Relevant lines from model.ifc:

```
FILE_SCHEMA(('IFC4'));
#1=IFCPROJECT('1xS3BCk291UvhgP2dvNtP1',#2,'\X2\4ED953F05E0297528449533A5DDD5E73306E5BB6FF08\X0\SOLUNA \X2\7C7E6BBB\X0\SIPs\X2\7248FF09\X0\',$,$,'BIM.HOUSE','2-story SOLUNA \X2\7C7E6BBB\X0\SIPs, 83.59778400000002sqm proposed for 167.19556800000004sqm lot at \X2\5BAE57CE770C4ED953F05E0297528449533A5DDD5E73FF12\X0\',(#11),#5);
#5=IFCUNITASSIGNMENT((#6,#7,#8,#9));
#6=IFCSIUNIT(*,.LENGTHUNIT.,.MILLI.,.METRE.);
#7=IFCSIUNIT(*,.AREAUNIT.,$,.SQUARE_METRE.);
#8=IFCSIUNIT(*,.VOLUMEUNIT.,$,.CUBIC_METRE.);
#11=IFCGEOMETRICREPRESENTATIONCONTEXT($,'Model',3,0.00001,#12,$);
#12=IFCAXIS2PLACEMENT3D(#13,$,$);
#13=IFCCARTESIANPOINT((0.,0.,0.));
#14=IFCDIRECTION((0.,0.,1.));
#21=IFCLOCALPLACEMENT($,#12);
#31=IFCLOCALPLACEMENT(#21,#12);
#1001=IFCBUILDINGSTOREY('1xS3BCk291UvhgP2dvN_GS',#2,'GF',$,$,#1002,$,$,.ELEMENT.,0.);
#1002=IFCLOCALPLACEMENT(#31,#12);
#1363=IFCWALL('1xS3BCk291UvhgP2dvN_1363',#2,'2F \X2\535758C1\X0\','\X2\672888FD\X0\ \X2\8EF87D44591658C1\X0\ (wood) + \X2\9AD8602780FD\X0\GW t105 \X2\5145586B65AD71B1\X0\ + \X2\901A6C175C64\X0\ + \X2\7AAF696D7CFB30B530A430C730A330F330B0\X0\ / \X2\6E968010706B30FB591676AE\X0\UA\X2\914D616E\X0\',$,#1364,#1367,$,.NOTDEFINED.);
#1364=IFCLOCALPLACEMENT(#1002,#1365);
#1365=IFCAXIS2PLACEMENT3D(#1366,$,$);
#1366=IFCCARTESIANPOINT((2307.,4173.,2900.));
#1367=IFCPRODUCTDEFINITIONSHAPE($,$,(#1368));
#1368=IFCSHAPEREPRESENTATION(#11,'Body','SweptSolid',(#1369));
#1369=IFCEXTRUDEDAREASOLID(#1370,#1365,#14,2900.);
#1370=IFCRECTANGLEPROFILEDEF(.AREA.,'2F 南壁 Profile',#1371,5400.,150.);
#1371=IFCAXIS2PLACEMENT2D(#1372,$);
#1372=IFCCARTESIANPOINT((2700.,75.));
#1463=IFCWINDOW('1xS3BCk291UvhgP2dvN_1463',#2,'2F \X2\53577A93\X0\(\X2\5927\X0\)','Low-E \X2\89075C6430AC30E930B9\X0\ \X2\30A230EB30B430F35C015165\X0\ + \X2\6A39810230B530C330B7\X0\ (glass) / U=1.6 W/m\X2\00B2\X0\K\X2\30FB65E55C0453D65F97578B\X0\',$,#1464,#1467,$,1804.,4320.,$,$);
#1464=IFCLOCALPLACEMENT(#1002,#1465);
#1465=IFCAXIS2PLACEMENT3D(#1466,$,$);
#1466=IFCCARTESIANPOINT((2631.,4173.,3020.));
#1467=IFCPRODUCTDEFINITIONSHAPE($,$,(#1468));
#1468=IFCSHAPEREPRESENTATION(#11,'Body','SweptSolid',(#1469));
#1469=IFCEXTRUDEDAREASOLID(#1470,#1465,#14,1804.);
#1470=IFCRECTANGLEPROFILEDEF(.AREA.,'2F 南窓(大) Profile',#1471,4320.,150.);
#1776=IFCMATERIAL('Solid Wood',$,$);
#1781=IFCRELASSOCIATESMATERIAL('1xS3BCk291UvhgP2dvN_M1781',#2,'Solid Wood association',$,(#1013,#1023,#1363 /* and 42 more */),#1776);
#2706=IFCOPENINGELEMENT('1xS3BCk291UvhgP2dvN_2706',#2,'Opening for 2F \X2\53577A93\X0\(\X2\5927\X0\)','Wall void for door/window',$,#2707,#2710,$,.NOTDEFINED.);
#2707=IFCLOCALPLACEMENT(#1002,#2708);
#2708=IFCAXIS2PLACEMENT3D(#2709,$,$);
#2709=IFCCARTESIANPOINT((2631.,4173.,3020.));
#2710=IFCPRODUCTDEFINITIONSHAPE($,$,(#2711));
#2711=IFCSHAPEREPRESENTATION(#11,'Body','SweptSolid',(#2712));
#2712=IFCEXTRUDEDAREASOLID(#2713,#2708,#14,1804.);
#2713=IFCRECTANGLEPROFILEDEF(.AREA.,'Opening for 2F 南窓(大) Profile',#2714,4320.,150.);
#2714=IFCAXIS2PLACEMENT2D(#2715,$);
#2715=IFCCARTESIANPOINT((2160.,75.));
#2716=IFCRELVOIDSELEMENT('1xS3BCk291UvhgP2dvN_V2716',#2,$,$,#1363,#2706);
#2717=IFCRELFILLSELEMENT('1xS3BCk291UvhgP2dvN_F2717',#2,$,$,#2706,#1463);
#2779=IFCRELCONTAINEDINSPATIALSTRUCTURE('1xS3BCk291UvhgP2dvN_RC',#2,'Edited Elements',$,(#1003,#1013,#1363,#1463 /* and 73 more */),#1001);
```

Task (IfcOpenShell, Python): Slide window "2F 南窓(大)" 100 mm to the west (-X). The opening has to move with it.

```python
import ifcopenshell
import ifcopenshell.api.geometry
import ifcopenshell.util.placement
import ifcopenshell.util.unit

model = ifcopenshell.open("model.ifc")
unit_scale = ifcopenshell.util.unit.calculate_unit_scale(model)

window = model.by_id(1463)
opening = window.FillsVoids[0].RelatingOpeningElement
wall = opening.VoidsElements[0].RelatingBuildingElement

wall_matrix = ifcopenshell.util.placement.get_local_placement(wall.ObjectPlacement)
shift = wall_matrix[:3, 0] * -0.1 / unit_scale
before = ifcopenshell.util.placement.get_local_placement(window.ObjectPlacement)[:3, 3].copy()

# The window is not placed relative to its opening, so move both.
for product in (opening, window):
    matrix = ifcopenshell.util.placement.get_local_placement(product.ObjectPlacement)
    matrix[:3, 3] += shift
    ifcopenshell.api.geometry.edit_object_placement(model, product=product, matrix=matrix, is_si=False)

after = ifcopenshell.util.placement.get_local_placement(window.ObjectPlacement)[:3, 3]
print("window moved by", (after - before).round(3) + 0.0)

model.write("model_v2.ifc")
```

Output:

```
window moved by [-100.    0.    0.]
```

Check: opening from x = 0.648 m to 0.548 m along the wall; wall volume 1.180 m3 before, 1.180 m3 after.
